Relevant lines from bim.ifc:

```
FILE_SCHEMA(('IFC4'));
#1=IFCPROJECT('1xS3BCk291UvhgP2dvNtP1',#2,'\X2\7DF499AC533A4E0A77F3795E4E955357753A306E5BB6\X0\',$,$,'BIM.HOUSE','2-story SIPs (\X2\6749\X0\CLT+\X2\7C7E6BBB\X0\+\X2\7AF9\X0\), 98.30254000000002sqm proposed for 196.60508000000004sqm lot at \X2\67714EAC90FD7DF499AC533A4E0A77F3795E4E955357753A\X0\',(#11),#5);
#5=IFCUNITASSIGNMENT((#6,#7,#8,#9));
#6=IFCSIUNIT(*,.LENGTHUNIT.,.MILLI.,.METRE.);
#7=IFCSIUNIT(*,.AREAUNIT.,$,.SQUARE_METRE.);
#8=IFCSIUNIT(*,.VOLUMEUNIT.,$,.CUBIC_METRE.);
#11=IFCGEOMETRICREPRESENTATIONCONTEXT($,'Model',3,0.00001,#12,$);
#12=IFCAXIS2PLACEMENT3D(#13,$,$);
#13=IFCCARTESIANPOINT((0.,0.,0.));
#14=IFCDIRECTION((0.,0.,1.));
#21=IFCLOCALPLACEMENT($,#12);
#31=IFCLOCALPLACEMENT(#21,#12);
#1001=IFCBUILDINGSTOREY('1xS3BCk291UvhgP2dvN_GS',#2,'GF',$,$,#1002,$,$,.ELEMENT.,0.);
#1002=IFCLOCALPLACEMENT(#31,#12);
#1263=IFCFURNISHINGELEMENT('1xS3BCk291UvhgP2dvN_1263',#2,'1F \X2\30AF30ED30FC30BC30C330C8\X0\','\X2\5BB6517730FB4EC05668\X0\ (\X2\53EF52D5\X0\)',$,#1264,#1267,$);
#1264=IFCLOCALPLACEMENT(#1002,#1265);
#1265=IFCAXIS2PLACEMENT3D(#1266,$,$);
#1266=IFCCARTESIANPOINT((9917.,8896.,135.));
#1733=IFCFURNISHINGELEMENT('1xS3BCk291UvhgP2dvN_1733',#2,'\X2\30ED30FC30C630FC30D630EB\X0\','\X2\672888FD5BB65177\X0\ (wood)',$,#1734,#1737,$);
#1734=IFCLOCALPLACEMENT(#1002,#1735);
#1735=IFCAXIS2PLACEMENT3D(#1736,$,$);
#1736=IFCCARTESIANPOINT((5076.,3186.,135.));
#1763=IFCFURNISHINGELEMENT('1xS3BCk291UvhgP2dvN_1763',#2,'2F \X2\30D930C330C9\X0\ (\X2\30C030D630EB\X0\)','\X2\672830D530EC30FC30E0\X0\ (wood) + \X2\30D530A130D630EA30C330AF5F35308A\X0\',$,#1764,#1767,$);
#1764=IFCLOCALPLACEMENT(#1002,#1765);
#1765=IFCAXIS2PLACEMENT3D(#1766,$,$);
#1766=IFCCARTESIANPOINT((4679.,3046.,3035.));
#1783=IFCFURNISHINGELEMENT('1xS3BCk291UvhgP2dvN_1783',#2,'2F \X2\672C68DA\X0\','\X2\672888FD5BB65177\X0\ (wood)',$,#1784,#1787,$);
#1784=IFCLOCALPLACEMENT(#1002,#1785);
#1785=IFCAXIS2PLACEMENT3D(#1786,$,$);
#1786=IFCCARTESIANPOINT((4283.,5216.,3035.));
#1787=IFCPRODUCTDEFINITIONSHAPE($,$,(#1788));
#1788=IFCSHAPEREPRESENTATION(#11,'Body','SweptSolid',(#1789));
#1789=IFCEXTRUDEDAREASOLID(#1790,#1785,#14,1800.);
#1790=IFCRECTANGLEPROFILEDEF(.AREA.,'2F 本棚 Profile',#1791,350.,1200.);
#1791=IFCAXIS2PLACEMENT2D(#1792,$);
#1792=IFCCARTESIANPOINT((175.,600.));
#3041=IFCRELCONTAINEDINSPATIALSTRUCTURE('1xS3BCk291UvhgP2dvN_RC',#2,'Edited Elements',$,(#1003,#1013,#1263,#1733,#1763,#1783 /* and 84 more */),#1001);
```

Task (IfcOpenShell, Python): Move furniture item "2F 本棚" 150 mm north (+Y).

```python
import ifcopenshell
import ifcopenshell.api.geometry
import ifcopenshell.util.placement

model = ifcopenshell.open("bim.ifc")

item = model.by_guid("1xS3BCk291UvhgP2dvN_1783")
matrix = ifcopenshell.util.placement.get_local_placement(item.ObjectPlacement)
matrix[1, 3] += 150.0
ifcopenshell.api.geometry.edit_object_placement(model, product=item, matrix=matrix, is_si=False)

print(ifcopenshell.util.placement.get_local_placement(item.ObjectPlacement).round(3) + 0.0)

model.write("bim_rev.ifc")
```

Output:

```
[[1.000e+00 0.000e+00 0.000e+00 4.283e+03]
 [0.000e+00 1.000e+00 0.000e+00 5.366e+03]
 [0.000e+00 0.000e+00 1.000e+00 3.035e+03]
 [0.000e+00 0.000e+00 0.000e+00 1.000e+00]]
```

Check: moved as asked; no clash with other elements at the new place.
